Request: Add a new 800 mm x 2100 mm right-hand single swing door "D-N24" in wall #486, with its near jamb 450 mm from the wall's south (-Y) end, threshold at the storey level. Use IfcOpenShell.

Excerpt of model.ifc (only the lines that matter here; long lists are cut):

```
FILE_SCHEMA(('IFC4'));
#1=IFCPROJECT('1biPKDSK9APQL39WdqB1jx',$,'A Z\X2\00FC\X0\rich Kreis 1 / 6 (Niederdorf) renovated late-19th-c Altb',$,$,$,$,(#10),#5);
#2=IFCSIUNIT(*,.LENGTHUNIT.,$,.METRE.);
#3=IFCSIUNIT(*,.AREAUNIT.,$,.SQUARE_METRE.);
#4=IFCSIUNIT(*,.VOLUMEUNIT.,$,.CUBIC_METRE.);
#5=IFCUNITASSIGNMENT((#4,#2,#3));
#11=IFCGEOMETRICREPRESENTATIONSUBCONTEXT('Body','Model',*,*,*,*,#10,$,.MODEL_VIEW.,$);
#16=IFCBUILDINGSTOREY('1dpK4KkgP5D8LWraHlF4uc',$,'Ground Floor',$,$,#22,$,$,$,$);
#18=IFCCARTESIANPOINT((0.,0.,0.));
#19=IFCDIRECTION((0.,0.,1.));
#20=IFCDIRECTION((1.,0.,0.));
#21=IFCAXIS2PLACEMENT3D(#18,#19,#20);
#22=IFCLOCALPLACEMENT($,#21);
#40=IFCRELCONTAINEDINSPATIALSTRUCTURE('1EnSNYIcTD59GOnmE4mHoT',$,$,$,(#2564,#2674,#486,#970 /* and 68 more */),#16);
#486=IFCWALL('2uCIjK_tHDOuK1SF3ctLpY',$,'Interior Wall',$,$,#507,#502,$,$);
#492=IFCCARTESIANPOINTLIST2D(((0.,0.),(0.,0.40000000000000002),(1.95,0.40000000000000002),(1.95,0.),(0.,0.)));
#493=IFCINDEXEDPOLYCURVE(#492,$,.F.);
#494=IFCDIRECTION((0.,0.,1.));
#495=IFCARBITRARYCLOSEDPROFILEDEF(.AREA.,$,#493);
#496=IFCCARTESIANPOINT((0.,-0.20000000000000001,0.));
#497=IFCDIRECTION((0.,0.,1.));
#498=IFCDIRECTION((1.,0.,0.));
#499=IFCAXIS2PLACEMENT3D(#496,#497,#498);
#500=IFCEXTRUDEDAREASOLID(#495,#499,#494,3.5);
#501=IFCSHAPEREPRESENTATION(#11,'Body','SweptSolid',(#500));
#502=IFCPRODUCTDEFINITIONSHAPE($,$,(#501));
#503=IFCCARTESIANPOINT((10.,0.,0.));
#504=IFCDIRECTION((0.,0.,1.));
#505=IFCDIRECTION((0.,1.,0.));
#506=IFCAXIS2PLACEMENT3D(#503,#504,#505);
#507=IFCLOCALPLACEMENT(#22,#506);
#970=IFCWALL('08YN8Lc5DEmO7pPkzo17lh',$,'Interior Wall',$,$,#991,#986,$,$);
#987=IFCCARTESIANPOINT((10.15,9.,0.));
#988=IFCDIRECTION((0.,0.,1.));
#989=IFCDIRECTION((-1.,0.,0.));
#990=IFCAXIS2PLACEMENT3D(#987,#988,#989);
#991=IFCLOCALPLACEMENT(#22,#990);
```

```python
import numpy as np
import ifcopenshell
import ifcopenshell.api.feature
import ifcopenshell.api.geometry
import ifcopenshell.api.root
import ifcopenshell.api.spatial
import ifcopenshell.geom
import ifcopenshell.util.element
import ifcopenshell.util.placement
import ifcopenshell.util.representation
import ifcopenshell.util.shape
import ifcopenshell.util.unit

model = ifcopenshell.open("model.ifc")
unit_scale = ifcopenshell.util.unit.calculate_unit_scale(model)
settings = ifcopenshell.geom.settings()


def volume(element):
    """Net volume in cubic metres, openings subtracted."""
    shape = ifcopenshell.geom.create_shape(settings, element)
    return ifcopenshell.util.shape.get_volume(shape.geometry)


wall = model.by_guid("2uCIjK_tHDOuK1SF3ctLpY")
storey = ifcopenshell.util.element.get_container(wall, ifc_class="IfcBuildingStorey")
context = ifcopenshell.util.representation.get_context(model, "Model", "Body", "MODEL_VIEW")
before = volume(wall)

width, height, from_end, sill = 0.8, 2.1, 0.45, 0.0  # metres

# The wall runs along its own X axis, and the end named is its -X end.
wall_shape = ifcopenshell.geom.create_shape(settings, wall)
x, y, z = ifcopenshell.util.shape.get_vertices(wall_shape.geometry).T
start = x.min() + from_end
face, thickness = float(y.min()), float(y.max() - y.min())
wall_matrix = ifcopenshell.util.placement.get_local_placement(wall.ObjectPlacement)
level = ifcopenshell.util.placement.get_local_placement(storey.ObjectPlacement)[2, 3]


def in_wall(x, y):
    """Placement at x, y metres in the wall's axes, at sill height."""
    matrix = wall_matrix.copy()
    matrix[:, 3] = wall_matrix @ np.array([x / unit_scale, y / unit_scale, 0.0, 1.0])
    matrix[2, 3] = level + sill / unit_scale
    return matrix


# Opening: a box that overshoots both wall faces by 50 mm.
opening = ifcopenshell.api.root.create_entity(model, ifc_class="IfcOpeningElement", predefined_type="OPENING")
box = ifcopenshell.api.geometry.add_wall_representation(
    model, context=context, length=width, height=height, thickness=thickness + 0.1
)
ifcopenshell.api.geometry.assign_representation(model, product=opening, representation=box)
ifcopenshell.api.geometry.edit_object_placement(model, product=opening, matrix=in_wall(start, face - 0.05), is_si=False)
ifcopenshell.api.feature.add_feature(model, feature=opening, element=wall)

door = ifcopenshell.api.root.create_entity(model, ifc_class="IfcDoor", name="D-N24", predefined_type="DOOR")
door.OverallWidth, door.OverallHeight = width / unit_scale, height / unit_scale
door.OperationType = "SINGLE_SWING_RIGHT"
body = ifcopenshell.api.geometry.add_door_representation(
    model,
    context=context,
    overall_width=door.OverallWidth,
    overall_height=door.OverallHeight,
    operation_type="SINGLE_SWING_RIGHT",
    lining_properties={"LiningDepth": thickness / unit_scale, "ThresholdDepth": thickness / unit_scale},
)
ifcopenshell.api.geometry.assign_representation(model, product=door, representation=body)
ifcopenshell.api.spatial.assign_container(model, products=[door], relating_structure=storey)
ifcopenshell.api.feature.add_filling(model, opening=opening, element=door)

# The lining spans the wall, so the door starts at the wall face.
ifcopenshell.api.geometry.edit_object_placement(model, product=door, matrix=in_wall(start, face), is_si=False)

after = volume(wall)

print(f"wall volume {before:.3f} -> {after:.3f} m3")

model.write("model_rev.ifc")
```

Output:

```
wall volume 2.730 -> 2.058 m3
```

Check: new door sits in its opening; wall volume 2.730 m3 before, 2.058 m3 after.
